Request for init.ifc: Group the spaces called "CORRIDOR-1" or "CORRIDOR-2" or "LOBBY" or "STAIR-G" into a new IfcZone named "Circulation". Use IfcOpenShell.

First a look at what the model holds.

```python
import ifcopenshell

model = ifcopenshell.open("init.ifc")
print(model.schema)
seen = {}
for space in model.by_type("IfcSpace"):
    seen[space.Name] = seen.get(space.Name, 0) + 1
for name, count in sorted(seen.items(), key=str):
    print(count, "x", name)
print("zones:", [z.Name for z in model.by_type("IfcZone")][:20])
```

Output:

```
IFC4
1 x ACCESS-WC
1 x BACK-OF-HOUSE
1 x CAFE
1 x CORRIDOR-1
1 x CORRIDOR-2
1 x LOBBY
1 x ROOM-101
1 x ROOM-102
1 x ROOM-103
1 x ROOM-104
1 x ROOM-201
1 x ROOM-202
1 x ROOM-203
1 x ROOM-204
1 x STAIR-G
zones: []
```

```python
import ifcopenshell
import ifcopenshell.api.group
import ifcopenshell.api.root

model = ifcopenshell.open("init.ifc")

names = {"CORRIDOR-1", "CORRIDOR-2", "LOBBY", "STAIR-G"}
spaces = [s for s in model.by_type("IfcSpace") if s.Name in names]

zone = ifcopenshell.api.root.create_entity(model, ifc_class="IfcZone", name="Circulation")
ifcopenshell.api.group.assign_group(model, products=spaces, group=zone)
print(len(spaces), "spaces in", zone.Name)

model.write("init_v2.ifc")
```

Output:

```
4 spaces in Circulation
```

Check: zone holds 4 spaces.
